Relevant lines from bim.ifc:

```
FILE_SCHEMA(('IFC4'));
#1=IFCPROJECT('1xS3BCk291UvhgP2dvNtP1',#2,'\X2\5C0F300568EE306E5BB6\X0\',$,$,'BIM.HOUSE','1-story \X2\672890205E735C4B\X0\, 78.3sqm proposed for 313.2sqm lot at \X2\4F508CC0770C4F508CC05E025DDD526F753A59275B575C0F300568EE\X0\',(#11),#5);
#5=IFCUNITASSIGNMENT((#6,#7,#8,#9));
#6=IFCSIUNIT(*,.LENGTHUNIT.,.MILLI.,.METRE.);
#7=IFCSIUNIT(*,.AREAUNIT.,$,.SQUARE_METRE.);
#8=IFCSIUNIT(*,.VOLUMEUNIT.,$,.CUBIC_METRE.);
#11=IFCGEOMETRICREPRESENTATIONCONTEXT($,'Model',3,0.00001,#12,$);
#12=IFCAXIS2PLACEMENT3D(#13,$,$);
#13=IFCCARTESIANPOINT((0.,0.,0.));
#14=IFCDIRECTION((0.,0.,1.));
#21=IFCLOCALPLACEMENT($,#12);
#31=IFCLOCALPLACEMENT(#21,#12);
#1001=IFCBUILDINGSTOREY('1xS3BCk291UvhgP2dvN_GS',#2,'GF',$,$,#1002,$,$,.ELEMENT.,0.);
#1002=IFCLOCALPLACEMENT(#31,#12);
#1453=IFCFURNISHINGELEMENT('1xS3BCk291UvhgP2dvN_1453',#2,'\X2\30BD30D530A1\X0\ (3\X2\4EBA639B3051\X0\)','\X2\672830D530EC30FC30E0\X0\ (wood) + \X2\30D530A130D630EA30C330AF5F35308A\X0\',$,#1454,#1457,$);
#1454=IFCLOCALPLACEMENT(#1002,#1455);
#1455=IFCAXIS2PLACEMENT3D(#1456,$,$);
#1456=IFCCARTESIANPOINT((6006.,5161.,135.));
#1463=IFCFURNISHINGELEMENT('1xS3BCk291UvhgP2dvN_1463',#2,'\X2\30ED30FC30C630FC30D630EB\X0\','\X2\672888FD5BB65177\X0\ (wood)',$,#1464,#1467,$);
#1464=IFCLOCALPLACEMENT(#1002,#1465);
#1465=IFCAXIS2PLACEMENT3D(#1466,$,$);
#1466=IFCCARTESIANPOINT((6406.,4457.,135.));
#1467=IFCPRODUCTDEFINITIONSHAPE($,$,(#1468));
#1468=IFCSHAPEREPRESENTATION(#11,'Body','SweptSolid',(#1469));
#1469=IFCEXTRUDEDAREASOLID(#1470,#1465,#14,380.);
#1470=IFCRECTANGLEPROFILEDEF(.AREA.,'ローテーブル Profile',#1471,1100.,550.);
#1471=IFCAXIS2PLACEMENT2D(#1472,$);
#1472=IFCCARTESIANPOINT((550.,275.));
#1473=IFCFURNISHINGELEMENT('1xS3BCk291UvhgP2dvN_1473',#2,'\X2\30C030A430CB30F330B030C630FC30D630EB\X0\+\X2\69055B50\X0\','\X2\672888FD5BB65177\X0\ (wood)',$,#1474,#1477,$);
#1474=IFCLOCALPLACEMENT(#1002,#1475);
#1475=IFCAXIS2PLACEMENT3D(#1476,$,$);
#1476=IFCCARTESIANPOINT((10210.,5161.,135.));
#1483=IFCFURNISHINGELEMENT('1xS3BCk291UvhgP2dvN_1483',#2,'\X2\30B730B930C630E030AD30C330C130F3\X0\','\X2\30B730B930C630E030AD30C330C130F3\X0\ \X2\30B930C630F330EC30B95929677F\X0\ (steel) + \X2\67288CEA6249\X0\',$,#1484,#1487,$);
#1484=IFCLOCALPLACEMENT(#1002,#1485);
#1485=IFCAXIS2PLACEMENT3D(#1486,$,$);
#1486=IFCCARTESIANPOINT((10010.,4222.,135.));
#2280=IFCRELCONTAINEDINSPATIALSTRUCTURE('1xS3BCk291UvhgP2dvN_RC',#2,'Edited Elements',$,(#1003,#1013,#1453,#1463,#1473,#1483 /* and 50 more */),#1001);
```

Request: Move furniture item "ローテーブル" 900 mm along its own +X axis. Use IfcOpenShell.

```python
import ifcopenshell
import ifcopenshell.api.geometry
import ifcopenshell.util.placement

model = ifcopenshell.open("bim.ifc")

item = model.by_guid("1xS3BCk291UvhgP2dvN_1463")
matrix = ifcopenshell.util.placement.get_local_placement(item.ObjectPlacement)
matrix[:3, 3] += matrix[:3, 0] * 900.0
ifcopenshell.api.geometry.edit_object_placement(model, product=item, matrix=matrix, is_si=False)

print(ifcopenshell.util.placement.get_local_placement(item.ObjectPlacement).round(3) + 0.0)

model.write("bim_edited.ifc")
```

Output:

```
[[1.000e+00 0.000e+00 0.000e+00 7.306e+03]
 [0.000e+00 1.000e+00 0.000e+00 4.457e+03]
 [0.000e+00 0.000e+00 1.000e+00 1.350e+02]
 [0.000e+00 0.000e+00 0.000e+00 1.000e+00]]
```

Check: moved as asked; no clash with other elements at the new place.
